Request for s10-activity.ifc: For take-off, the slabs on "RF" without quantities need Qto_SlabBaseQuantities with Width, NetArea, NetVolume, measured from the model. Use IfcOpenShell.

First a look at what the model holds.

```python
import ifcopenshell
import ifcopenshell.util.element
import ifcopenshell.util.unit

model = ifcopenshell.open("s10-activity.ifc")
print(model.schema)
for unit_type in ("LENGTHUNIT", "AREAUNIT", "VOLUMEUNIT"):
    print(unit_type, ifcopenshell.util.unit.calculate_unit_scale(model, unit_type))
storey = next(s for s in model.by_type("IfcBuildingStorey") if s.Name == "RF")
slabs = [e for e in ifcopenshell.util.element.get_decomposition(storey) if e.is_a("IfcSlab")]
for e in sorted(slabs, key=lambda e: e.id()):
    print(e.id(), e.is_a(), e.Name, list(ifcopenshell.util.element.get_psets(e, qtos_only=True)), sep=" | ")
```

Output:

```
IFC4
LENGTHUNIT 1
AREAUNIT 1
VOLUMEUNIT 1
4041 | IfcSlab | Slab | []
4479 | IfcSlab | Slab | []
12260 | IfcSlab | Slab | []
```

```python
import ifcopenshell
import ifcopenshell.api.pset
import ifcopenshell.geom
import ifcopenshell.util.element
import ifcopenshell.util.shape
import ifcopenshell.util.unit

model = ifcopenshell.open("s10-activity.ifc")
unit_scale = ifcopenshell.util.unit.calculate_unit_scale(model)
area_scale = ifcopenshell.util.unit.calculate_unit_scale(model, "AREAUNIT")
volume_scale = ifcopenshell.util.unit.calculate_unit_scale(model, "VOLUMEUNIT")
settings = ifcopenshell.geom.settings()

storey = next(s for s in model.by_type("IfcBuildingStorey") if s.Name == "RF")
slabs = [e for e in ifcopenshell.util.element.get_decomposition(storey) if e.is_a("IfcSlab")]

for e in sorted(slabs, key=lambda e: e.id()):
    if ifcopenshell.util.element.get_psets(e, qtos_only=True, should_inherit=False):
        continue
    # Geometry comes back in metres, in the element's own axes.
    shape = ifcopenshell.geom.create_shape(settings, e)
    values = {
        "Width": ifcopenshell.util.shape.get_z(shape.geometry) / unit_scale,
        "NetArea": ifcopenshell.util.shape.get_footprint_area(shape.geometry) / area_scale,
        "NetVolume": ifcopenshell.util.shape.get_volume(shape.geometry) / volume_scale,
    }
    qto = ifcopenshell.api.pset.add_qto(model, product=e, name="Qto_SlabBaseQuantities")
    ifcopenshell.api.pset.edit_qto(model, qto=qto, properties=values)
    print(e.id(), {k: round(v, 3) for k, v in values.items()})

model.write("s10-activity_updated.ifc")
```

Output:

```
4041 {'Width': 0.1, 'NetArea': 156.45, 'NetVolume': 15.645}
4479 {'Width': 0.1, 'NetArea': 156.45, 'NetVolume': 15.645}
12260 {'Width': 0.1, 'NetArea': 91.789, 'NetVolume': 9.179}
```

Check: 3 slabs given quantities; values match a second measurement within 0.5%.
